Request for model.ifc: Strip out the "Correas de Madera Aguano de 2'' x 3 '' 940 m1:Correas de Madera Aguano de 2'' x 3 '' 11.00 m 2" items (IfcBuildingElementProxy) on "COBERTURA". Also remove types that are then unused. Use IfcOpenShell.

First a look at what the model holds.

```python
import ifcopenshell
import ifcopenshell.util.element

model = ifcopenshell.open("model.ifc")
print(model.schema)
storey = next(s for s in model.by_type("IfcBuildingStorey") if s.Name == "COBERTURA")
proxies = [e for e in ifcopenshell.util.element.get_decomposition(storey) if e.is_a("IfcBuildingElementProxy")]
seen = {}
for e in proxies:
    element_type = ifcopenshell.util.element.get_type(e)
    name = element_type.Name if element_type not in (None, e) else None
    seen[name] = seen.get(name, 0) + 1
for name, count in sorted(seen.items(), key=str):
    print(count, "x", name)
```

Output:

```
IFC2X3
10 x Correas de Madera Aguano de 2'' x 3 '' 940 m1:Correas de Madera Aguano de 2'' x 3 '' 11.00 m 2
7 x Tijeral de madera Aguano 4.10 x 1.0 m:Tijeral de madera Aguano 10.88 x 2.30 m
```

```python
import ifcopenshell
import ifcopenshell.api.root
import ifcopenshell.util.element

model = ifcopenshell.open("model.ifc")

storey = next(s for s in model.by_type("IfcBuildingStorey") if s.Name == "COBERTURA")
proxies = [e for e in ifcopenshell.util.element.get_decomposition(storey) if e.is_a("IfcBuildingElementProxy")]
targets = [e for e in proxies if (t := ifcopenshell.util.element.get_type(e)) not in (None, e) and t.Name == "Correas de Madera Aguano de 2'' x 3 '' 940 m1:Correas de Madera Aguano de 2'' x 3 '' 11.00 m 2"]
types = {ifcopenshell.util.element.get_type(e) for e in targets} - {None, *targets}

for e in targets:
    ifcopenshell.api.root.remove_product(model, product=e)
print(len(targets), "removed")

unused = [t for t in types if not ifcopenshell.util.element.get_types(t)]
for t in unused:
    ifcopenshell.api.root.remove_product(model, product=t)
print(len(unused), "unused types removed")

model.write("model_edited.ifc")
```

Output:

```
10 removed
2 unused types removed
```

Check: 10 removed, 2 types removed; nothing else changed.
